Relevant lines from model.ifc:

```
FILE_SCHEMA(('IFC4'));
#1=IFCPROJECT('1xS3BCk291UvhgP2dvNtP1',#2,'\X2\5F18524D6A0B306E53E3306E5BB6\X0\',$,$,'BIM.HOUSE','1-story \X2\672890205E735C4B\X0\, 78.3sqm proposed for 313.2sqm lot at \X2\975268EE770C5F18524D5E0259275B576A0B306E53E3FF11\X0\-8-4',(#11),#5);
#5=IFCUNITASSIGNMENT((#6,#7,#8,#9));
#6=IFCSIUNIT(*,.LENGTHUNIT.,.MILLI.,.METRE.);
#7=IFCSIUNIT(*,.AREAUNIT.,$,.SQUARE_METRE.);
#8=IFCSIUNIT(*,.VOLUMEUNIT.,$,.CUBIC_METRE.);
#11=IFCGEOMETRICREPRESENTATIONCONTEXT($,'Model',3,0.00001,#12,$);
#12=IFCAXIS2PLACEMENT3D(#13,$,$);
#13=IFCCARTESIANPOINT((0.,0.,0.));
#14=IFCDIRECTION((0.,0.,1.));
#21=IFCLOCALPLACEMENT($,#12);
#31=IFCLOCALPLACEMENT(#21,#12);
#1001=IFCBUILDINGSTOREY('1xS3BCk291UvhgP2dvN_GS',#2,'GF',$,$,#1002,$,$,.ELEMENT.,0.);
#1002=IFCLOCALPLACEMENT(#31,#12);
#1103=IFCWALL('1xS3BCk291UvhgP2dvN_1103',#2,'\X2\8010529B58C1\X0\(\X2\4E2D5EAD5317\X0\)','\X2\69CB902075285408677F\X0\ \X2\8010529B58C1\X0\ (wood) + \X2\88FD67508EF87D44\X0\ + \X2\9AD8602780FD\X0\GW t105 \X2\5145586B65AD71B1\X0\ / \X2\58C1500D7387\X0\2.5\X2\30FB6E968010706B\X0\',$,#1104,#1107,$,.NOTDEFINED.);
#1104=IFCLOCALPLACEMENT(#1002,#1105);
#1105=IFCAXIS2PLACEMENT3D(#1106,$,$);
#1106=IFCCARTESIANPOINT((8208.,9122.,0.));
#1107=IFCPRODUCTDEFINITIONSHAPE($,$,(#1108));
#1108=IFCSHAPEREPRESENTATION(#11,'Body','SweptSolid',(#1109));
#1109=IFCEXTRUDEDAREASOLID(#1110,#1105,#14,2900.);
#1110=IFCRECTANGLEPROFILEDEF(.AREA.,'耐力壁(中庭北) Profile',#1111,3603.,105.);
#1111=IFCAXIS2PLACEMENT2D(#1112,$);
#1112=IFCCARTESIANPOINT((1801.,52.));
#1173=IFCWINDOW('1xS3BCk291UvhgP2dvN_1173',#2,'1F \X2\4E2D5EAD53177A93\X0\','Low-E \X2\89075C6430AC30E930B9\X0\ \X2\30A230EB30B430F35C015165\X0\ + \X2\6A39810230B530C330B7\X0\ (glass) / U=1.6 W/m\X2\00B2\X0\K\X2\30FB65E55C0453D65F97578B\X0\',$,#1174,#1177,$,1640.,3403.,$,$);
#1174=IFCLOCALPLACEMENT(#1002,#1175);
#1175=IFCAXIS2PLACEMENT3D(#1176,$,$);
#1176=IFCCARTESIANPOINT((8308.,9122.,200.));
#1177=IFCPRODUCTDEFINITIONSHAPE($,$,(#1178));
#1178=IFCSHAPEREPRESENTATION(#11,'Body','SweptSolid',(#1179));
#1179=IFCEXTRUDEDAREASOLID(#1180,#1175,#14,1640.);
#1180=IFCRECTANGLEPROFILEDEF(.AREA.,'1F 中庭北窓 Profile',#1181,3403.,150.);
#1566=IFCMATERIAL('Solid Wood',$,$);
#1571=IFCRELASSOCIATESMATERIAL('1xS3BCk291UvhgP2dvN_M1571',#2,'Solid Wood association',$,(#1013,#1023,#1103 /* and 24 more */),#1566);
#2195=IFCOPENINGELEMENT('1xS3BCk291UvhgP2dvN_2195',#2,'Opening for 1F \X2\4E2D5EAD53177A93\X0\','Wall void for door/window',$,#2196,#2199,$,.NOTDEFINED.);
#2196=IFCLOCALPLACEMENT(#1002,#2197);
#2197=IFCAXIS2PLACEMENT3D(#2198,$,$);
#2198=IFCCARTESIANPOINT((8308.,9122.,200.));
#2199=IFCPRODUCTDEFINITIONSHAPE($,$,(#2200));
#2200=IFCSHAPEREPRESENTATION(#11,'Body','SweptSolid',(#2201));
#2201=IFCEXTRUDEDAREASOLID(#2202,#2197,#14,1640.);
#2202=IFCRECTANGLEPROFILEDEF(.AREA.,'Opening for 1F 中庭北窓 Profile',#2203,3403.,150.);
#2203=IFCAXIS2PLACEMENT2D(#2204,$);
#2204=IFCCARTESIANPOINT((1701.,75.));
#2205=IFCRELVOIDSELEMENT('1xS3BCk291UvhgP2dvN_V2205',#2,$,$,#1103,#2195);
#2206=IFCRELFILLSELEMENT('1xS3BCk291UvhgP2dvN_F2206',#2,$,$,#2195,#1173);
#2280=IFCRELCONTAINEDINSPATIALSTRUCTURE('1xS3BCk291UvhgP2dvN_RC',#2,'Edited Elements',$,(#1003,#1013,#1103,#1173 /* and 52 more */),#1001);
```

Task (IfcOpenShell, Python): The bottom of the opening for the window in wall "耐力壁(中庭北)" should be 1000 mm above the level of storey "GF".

```python
import numpy as np
import ifcopenshell
import ifcopenshell.api.geometry
import ifcopenshell.geom
import ifcopenshell.util.element
import ifcopenshell.util.placement
import ifcopenshell.util.shape
import ifcopenshell.util.unit

model = ifcopenshell.open("model.ifc")
unit_scale = ifcopenshell.util.unit.calculate_unit_scale(model)

window = model.by_id(1173)
opening = window.FillsVoids[0].RelatingOpeningElement
storey = ifcopenshell.util.element.get_container(window, ifc_class="IfcBuildingStorey")
level = ifcopenshell.util.placement.get_local_placement(storey.ObjectPlacement)[2, 3]

# The opening's origin need not be at the sill, so measure its lowest point.
shape = ifcopenshell.geom.create_shape(ifcopenshell.geom.settings(), opening)
bottom = ifcopenshell.util.shape.get_shape_bottom_elevation(shape, shape.geometry) / unit_scale
dz = level + 1000.0 - bottom

shift = np.array([0.0, 0.0, dz])
# The window is not placed relative to its opening, so move both.
for product in (opening, window):
    matrix = ifcopenshell.util.placement.get_local_placement(product.ObjectPlacement)
    matrix[:3, 3] += shift
    ifcopenshell.api.geometry.edit_object_placement(model, product=product, matrix=matrix, is_si=False)

print(f"moved by {dz * unit_scale:+.3f} m")

model.write("model_updated.ifc")
```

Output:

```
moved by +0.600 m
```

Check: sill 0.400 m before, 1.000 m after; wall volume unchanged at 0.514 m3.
